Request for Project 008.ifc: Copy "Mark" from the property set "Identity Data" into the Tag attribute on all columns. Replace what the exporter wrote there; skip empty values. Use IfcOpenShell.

First a look at what the model holds.

```python
import ifcopenshell
import ifcopenshell.util.element

model = ifcopenshell.open("Project 008.ifc")
print(model.schema)
columns = model.by_type("IfcColumn")
print(len(columns), "columns")
for e in columns[:8]:
    source = ifcopenshell.util.element.get_pset(e, "Identity Data", "Mark")
    target = e.Tag
    print(e.id(), repr(source), repr(target), sep=" | ")
```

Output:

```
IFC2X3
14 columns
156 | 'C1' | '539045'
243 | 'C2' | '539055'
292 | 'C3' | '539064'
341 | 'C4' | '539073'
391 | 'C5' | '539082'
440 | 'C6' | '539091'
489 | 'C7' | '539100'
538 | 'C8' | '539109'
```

```python
import ifcopenshell
import ifcopenshell.util.element

model = ifcopenshell.open("Project 008.ifc")

count = 0
for e in model.by_type("IfcColumn"):
    value = ifcopenshell.util.element.get_pset(e, "Identity Data", "Mark")
    current = e.Tag
    if not value or not value.strip() or current == value:
        continue
    e.Tag = value
    count += 1

print(count, "columns updated")

model.write("Project 008_updated.ifc")
```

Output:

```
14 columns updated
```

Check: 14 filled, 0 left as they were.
